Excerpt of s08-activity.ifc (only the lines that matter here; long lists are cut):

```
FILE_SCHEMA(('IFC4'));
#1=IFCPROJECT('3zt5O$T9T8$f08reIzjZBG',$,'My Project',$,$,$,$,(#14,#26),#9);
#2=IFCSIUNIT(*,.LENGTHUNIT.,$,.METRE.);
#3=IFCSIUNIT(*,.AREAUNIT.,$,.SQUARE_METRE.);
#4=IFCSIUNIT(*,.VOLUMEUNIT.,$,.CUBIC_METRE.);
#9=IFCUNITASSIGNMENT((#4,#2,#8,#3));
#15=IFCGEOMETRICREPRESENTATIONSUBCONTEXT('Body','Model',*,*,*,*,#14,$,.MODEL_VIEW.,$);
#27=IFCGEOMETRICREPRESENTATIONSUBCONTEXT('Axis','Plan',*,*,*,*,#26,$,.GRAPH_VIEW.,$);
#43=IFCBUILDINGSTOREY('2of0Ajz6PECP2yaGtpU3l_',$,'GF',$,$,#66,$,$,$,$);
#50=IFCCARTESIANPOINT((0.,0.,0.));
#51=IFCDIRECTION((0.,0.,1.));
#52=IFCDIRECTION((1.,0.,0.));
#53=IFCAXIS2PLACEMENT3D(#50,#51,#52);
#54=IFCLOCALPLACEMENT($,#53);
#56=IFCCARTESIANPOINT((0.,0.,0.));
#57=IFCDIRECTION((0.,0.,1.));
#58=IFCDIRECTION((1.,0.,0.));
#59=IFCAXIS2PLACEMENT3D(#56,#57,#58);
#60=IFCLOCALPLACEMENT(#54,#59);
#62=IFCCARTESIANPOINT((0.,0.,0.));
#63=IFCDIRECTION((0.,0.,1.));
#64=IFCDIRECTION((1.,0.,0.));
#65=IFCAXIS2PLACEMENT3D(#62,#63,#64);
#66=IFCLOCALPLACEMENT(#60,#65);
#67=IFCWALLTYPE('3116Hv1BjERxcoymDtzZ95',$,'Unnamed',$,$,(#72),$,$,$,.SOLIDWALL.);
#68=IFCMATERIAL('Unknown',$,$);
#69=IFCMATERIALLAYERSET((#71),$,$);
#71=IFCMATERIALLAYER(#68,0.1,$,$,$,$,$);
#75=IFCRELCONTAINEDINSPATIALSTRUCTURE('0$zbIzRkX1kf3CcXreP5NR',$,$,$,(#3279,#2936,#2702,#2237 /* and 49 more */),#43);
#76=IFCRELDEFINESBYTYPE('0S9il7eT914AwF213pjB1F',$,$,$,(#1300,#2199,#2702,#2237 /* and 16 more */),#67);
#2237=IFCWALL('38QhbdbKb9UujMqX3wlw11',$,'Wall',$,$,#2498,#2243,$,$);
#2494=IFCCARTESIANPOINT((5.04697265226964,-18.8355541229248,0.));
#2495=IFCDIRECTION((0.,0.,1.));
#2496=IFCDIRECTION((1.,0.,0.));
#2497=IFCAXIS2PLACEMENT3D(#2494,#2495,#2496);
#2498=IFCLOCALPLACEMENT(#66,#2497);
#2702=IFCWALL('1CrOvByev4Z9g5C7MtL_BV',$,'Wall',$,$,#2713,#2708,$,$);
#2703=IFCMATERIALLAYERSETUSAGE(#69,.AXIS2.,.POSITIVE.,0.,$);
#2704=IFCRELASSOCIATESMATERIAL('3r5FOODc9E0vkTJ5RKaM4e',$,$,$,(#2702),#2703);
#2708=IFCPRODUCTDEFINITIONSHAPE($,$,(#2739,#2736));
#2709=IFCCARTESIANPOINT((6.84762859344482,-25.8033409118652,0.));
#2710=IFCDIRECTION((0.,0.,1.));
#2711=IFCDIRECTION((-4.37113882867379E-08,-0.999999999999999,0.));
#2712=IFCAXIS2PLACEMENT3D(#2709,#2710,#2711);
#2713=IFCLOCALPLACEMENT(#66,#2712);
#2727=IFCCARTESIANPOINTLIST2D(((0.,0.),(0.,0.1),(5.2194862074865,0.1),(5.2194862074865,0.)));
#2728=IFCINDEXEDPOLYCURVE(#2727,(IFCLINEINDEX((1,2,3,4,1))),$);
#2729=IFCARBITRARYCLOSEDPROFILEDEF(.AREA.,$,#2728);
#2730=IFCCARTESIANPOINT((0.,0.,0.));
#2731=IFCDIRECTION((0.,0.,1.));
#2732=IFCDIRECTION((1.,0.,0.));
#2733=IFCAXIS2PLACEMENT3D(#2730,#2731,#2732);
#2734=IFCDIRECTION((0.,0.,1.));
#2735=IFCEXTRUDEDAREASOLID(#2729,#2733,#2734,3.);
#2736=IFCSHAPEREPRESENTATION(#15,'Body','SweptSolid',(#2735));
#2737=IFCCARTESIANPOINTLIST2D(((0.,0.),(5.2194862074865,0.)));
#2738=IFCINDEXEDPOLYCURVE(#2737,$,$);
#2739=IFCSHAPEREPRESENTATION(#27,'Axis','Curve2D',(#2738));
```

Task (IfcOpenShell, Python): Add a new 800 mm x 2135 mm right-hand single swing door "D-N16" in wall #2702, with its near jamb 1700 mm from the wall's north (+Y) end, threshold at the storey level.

```python
import numpy as np
import ifcopenshell
import ifcopenshell.api.feature
import ifcopenshell.api.geometry
import ifcopenshell.api.root
import ifcopenshell.api.spatial
import ifcopenshell.geom
import ifcopenshell.util.element
import ifcopenshell.util.placement
import ifcopenshell.util.representation
import ifcopenshell.util.shape
import ifcopenshell.util.unit

model = ifcopenshell.open("s08-activity.ifc")
unit_scale = ifcopenshell.util.unit.calculate_unit_scale(model)
settings = ifcopenshell.geom.settings()


def volume(element):
    """Net volume in cubic metres, openings subtracted."""
    shape = ifcopenshell.geom.create_shape(settings, element)
    return ifcopenshell.util.shape.get_volume(shape.geometry)


wall = model.by_guid("1CrOvByev4Z9g5C7MtL_BV")
storey = ifcopenshell.util.element.get_container(wall, ifc_class="IfcBuildingStorey")
context = ifcopenshell.util.representation.get_context(model, "Model", "Body", "MODEL_VIEW")
before = volume(wall)

width, height, from_end, sill = 0.8, 2.135, 1.7, 0.0  # metres

# The wall runs along its own X axis, and the end named is its -X end.
wall_shape = ifcopenshell.geom.create_shape(settings, wall)
x, y, z = ifcopenshell.util.shape.get_vertices(wall_shape.geometry).T
start = x.min() + from_end
face, thickness = float(y.min()), float(y.max() - y.min())
wall_matrix = ifcopenshell.util.placement.get_local_placement(wall.ObjectPlacement)
level = ifcopenshell.util.placement.get_local_placement(storey.ObjectPlacement)[2, 3]


def in_wall(x, y):
    """Placement at x, y metres in the wall's axes, at sill height."""
    matrix = wall_matrix.copy()
    matrix[:, 3] = wall_matrix @ np.array([x / unit_scale, y / unit_scale, 0.0, 1.0])
    matrix[2, 3] = level + sill / unit_scale
    return matrix


# Opening: a box that overshoots both wall faces by 50 mm.
opening = ifcopenshell.api.root.create_entity(model, ifc_class="IfcOpeningElement", predefined_type="OPENING")
box = ifcopenshell.api.geometry.add_wall_representation(
    model, context=context, length=width, height=height, thickness=thickness + 0.1
)
ifcopenshell.api.geometry.assign_representation(model, product=opening, representation=box)
ifcopenshell.api.geometry.edit_object_placement(model, product=opening, matrix=in_wall(start, face - 0.05), is_si=False)
ifcopenshell.api.feature.add_feature(model, feature=opening, element=wall)

door = ifcopenshell.api.root.create_entity(model, ifc_class="IfcDoor", name="D-N16", predefined_type="DOOR")
door.OverallWidth, door.OverallHeight = width / unit_scale, height / unit_scale
door.OperationType = "SINGLE_SWING_RIGHT"
body = ifcopenshell.api.geometry.add_door_representation(
    model,
    context=context,
    overall_width=door.OverallWidth,
    overall_height=door.OverallHeight,
    operation_type="SINGLE_SWING_RIGHT",
    lining_properties={"LiningDepth": thickness / unit_scale, "ThresholdDepth": thickness / unit_scale},
)
ifcopenshell.api.geometry.assign_representation(model, product=door, representation=body)
ifcopenshell.api.spatial.assign_container(model, products=[door], relating_structure=storey)
ifcopenshell.api.feature.add_filling(model, opening=opening, element=door)

# The lining spans the wall, so the door starts at the wall face.
ifcopenshell.api.geometry.edit_object_placement(model, product=door, matrix=in_wall(start, face), is_si=False)

after = volume(wall)

print(f"wall volume {before:.3f} -> {after:.3f} m3")

model.write("s08-activity_rev.ifc")
```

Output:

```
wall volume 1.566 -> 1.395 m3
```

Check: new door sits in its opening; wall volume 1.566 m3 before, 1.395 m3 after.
